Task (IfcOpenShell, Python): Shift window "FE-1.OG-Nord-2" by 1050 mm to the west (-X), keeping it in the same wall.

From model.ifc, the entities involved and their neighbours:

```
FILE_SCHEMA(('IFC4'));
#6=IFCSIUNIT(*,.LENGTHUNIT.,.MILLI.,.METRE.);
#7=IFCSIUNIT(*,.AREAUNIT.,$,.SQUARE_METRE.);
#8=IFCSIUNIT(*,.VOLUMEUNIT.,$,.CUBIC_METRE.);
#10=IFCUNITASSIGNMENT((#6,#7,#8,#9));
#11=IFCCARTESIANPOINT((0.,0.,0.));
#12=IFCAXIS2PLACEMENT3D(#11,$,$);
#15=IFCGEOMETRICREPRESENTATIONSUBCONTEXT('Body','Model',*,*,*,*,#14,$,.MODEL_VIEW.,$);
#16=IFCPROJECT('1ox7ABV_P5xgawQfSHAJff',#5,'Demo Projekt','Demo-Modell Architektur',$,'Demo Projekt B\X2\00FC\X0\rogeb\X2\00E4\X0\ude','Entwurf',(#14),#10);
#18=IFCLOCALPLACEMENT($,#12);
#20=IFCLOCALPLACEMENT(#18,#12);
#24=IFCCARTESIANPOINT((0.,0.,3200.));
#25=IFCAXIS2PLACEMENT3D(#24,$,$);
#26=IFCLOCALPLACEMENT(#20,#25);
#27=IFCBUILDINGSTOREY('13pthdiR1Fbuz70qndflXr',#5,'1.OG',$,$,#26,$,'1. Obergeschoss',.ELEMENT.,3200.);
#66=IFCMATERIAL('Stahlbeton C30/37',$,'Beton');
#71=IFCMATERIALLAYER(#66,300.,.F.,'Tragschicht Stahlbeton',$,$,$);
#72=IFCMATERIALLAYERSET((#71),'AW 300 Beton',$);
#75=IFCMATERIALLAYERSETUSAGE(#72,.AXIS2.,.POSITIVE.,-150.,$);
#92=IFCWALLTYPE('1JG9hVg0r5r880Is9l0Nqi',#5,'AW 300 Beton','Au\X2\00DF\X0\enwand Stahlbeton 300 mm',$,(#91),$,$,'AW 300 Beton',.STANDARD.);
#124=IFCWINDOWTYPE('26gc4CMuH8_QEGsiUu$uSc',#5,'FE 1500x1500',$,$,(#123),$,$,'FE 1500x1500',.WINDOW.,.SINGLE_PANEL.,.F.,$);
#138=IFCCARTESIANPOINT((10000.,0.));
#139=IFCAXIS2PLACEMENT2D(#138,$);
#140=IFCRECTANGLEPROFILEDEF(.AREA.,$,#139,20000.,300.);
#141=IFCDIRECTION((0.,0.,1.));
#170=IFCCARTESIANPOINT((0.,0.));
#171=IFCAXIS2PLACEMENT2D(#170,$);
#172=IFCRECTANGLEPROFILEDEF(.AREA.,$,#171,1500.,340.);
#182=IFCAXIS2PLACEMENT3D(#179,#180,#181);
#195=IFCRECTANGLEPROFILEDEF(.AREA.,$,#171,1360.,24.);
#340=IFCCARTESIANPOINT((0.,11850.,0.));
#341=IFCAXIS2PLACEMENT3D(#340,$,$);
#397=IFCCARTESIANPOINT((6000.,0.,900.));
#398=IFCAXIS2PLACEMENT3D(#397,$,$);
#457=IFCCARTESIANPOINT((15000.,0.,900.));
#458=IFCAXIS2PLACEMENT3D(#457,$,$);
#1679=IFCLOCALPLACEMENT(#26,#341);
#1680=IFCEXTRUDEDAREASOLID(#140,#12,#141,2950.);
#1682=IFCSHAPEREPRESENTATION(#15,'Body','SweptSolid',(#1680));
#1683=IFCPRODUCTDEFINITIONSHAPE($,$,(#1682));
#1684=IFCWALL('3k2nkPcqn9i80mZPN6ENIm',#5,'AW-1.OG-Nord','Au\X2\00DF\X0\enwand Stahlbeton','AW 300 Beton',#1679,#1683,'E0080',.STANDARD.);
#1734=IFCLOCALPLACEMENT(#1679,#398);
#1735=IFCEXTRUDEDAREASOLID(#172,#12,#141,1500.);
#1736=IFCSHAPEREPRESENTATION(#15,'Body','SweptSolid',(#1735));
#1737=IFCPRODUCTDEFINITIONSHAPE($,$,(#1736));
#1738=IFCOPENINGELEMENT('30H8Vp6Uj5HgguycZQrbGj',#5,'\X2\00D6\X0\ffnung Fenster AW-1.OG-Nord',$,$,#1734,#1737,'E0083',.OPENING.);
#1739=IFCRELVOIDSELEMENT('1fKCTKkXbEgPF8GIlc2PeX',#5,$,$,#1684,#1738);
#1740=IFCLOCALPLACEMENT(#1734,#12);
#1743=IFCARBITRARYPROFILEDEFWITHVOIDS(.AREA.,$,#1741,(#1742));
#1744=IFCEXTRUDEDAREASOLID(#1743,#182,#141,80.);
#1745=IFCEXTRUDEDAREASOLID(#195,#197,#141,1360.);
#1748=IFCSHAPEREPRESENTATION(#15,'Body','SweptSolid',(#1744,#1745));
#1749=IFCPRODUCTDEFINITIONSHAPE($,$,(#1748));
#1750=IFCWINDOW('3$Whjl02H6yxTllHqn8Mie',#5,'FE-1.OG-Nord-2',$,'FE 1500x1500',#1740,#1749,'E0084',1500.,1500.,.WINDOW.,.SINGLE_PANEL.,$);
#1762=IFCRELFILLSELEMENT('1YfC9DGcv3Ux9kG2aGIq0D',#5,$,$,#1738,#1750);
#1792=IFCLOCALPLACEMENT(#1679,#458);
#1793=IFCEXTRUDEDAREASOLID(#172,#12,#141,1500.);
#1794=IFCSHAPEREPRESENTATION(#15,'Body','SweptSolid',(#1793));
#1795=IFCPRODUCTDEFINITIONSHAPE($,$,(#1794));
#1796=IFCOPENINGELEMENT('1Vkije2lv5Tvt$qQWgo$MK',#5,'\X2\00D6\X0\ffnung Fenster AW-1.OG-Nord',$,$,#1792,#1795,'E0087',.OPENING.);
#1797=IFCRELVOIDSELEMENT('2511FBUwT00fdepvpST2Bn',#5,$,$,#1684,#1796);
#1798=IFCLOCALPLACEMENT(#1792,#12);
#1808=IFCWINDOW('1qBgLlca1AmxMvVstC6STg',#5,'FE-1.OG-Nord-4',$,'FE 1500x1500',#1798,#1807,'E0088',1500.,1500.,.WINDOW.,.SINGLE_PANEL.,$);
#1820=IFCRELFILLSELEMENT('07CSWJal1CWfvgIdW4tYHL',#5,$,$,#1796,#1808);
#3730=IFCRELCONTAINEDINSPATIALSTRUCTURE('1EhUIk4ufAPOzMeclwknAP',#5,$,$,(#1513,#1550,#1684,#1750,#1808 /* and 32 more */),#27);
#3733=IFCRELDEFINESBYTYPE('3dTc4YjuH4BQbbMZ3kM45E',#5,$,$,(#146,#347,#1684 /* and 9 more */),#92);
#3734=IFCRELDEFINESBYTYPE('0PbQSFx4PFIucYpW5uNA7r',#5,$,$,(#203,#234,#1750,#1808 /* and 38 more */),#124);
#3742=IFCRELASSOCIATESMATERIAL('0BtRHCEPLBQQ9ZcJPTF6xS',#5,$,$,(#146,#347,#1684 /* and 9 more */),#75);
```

```python
import ifcopenshell
import ifcopenshell.api.geometry
import ifcopenshell.util.placement
import ifcopenshell.util.unit

model = ifcopenshell.open("model.ifc")
unit_scale = ifcopenshell.util.unit.calculate_unit_scale(model)

window = model.by_guid("3$Whjl02H6yxTllHqn8Mie")
opening = window.FillsVoids[0].RelatingOpeningElement
wall = opening.VoidsElements[0].RelatingBuildingElement

wall_matrix = ifcopenshell.util.placement.get_local_placement(wall.ObjectPlacement)
shift = wall_matrix[:3, 0] * -1.05 / unit_scale
before = ifcopenshell.util.placement.get_local_placement(window.ObjectPlacement)[:3, 3].copy()

# The window is placed relative to its opening, so it follows when the opening moves.
matrix = ifcopenshell.util.placement.get_local_placement(opening.ObjectPlacement)
matrix[:3, 3] += shift
ifcopenshell.api.geometry.edit_object_placement(
    model, product=opening, matrix=matrix, is_si=False, should_transform_children=True
)

after = ifcopenshell.util.placement.get_local_placement(window.ObjectPlacement)[:3, 3]
print("window moved by", (after - before).round(3) + 0.0)

model.write("model-out.ifc")
```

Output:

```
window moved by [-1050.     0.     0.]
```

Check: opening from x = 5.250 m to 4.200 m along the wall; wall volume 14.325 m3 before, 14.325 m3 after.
